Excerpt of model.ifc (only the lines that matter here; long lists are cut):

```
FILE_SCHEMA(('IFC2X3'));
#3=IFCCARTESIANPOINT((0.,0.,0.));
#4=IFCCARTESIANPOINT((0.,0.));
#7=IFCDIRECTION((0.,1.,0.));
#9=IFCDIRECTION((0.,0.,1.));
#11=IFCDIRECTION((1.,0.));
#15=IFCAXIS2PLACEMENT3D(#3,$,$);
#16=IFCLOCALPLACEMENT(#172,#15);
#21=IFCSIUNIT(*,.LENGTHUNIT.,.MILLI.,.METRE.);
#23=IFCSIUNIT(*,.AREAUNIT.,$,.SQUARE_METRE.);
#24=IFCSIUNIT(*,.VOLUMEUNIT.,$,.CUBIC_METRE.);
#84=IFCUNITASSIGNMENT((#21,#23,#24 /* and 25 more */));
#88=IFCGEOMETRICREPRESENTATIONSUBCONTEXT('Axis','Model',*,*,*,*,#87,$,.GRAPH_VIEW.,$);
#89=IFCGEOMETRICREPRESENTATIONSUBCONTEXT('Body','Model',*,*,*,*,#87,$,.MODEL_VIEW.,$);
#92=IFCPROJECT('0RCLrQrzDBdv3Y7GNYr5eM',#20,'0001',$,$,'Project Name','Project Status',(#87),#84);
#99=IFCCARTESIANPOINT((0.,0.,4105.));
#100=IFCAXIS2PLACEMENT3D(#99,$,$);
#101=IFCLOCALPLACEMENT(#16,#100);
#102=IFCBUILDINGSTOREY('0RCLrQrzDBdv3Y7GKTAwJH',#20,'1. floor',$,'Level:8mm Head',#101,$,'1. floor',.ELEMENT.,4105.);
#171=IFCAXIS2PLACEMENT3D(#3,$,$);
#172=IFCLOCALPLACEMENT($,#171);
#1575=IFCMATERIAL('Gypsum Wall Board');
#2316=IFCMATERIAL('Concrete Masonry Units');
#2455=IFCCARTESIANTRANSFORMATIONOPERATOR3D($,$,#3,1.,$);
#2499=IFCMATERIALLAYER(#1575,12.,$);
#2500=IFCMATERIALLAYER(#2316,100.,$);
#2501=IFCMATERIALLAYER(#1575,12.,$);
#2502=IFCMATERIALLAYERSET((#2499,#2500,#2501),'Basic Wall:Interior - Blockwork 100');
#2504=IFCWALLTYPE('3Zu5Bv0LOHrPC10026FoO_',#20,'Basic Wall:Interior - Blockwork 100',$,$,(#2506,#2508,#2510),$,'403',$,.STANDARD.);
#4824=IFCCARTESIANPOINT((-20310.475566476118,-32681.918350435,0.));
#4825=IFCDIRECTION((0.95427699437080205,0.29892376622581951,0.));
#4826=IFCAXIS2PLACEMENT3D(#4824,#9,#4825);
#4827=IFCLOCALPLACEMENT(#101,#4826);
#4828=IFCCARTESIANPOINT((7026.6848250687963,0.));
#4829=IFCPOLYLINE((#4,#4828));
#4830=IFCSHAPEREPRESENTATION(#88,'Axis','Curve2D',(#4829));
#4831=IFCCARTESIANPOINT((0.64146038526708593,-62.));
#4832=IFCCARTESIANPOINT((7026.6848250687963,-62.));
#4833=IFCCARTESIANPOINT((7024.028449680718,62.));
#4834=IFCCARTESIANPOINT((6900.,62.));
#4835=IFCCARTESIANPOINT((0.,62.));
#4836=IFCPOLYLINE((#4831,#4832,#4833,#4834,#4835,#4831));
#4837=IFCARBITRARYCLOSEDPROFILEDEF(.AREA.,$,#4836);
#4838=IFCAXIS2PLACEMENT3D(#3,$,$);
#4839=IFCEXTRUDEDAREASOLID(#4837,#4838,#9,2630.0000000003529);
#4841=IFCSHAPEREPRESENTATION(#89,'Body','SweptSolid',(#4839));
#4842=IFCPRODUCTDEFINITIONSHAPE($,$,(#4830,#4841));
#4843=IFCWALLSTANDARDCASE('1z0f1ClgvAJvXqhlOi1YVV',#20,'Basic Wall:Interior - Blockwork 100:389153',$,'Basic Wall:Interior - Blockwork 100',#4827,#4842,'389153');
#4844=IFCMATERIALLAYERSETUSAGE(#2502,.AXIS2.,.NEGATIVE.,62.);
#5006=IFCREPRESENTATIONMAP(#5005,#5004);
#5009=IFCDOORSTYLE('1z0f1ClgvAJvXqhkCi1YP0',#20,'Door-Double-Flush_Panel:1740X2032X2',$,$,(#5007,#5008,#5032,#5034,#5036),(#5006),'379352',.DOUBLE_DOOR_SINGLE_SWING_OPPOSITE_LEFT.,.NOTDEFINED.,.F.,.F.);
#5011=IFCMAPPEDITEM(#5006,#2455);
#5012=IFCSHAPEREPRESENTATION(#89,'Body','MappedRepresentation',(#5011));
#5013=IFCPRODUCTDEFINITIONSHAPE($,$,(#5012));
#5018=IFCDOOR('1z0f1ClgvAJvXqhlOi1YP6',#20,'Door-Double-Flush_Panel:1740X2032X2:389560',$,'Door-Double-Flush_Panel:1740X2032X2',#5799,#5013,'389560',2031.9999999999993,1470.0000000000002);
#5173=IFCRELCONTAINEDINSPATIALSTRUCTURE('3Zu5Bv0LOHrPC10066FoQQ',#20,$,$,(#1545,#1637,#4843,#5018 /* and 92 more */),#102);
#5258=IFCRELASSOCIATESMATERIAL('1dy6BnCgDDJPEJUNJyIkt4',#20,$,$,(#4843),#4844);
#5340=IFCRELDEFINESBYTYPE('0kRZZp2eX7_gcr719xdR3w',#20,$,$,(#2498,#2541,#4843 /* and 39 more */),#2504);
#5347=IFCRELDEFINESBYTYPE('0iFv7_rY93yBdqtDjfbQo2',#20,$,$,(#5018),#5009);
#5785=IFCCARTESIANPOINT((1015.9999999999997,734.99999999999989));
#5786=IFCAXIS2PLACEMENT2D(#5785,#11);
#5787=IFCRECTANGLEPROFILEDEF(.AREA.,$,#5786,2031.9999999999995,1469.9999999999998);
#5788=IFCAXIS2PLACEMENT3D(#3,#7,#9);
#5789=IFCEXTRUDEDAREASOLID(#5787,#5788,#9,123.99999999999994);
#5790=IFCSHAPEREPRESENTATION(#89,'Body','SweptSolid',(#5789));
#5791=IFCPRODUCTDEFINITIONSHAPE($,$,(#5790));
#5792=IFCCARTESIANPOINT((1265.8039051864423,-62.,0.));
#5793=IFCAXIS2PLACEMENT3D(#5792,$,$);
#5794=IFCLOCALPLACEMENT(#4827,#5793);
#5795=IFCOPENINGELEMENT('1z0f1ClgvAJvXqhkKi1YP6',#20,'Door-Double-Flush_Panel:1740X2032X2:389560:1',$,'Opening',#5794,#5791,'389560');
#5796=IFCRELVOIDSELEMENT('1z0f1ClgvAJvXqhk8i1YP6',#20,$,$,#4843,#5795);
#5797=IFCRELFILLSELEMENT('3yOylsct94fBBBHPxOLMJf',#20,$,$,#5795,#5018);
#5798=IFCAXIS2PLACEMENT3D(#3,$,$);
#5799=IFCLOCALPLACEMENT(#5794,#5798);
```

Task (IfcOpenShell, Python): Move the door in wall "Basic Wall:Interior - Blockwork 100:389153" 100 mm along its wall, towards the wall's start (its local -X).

```python
import ifcopenshell
import ifcopenshell.api.geometry
import ifcopenshell.util.placement

model = ifcopenshell.open("model.ifc")

door = model.by_guid("1z0f1ClgvAJvXqhlOi1YP6")
opening = door.FillsVoids[0].RelatingOpeningElement
wall = opening.VoidsElements[0].RelatingBuildingElement

wall_matrix = ifcopenshell.util.placement.get_local_placement(wall.ObjectPlacement)
shift = wall_matrix[:3, 0] * -100.0
before = ifcopenshell.util.placement.get_local_placement(door.ObjectPlacement)[:3, 3].copy()

# The door is placed relative to its opening, so it follows when the opening moves.
matrix = ifcopenshell.util.placement.get_local_placement(opening.ObjectPlacement)
matrix[:3, 3] += shift
ifcopenshell.api.geometry.edit_object_placement(
    model, product=opening, matrix=matrix, is_si=False, should_transform_children=True
)

after = ifcopenshell.util.placement.get_local_placement(door.ObjectPlacement)[:3, 3]
print("door moved by", (after - before).round(3) + 0.0)

model.write("model-out.ifc")
```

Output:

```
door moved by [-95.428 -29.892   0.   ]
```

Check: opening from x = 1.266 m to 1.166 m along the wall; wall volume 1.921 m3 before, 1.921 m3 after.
